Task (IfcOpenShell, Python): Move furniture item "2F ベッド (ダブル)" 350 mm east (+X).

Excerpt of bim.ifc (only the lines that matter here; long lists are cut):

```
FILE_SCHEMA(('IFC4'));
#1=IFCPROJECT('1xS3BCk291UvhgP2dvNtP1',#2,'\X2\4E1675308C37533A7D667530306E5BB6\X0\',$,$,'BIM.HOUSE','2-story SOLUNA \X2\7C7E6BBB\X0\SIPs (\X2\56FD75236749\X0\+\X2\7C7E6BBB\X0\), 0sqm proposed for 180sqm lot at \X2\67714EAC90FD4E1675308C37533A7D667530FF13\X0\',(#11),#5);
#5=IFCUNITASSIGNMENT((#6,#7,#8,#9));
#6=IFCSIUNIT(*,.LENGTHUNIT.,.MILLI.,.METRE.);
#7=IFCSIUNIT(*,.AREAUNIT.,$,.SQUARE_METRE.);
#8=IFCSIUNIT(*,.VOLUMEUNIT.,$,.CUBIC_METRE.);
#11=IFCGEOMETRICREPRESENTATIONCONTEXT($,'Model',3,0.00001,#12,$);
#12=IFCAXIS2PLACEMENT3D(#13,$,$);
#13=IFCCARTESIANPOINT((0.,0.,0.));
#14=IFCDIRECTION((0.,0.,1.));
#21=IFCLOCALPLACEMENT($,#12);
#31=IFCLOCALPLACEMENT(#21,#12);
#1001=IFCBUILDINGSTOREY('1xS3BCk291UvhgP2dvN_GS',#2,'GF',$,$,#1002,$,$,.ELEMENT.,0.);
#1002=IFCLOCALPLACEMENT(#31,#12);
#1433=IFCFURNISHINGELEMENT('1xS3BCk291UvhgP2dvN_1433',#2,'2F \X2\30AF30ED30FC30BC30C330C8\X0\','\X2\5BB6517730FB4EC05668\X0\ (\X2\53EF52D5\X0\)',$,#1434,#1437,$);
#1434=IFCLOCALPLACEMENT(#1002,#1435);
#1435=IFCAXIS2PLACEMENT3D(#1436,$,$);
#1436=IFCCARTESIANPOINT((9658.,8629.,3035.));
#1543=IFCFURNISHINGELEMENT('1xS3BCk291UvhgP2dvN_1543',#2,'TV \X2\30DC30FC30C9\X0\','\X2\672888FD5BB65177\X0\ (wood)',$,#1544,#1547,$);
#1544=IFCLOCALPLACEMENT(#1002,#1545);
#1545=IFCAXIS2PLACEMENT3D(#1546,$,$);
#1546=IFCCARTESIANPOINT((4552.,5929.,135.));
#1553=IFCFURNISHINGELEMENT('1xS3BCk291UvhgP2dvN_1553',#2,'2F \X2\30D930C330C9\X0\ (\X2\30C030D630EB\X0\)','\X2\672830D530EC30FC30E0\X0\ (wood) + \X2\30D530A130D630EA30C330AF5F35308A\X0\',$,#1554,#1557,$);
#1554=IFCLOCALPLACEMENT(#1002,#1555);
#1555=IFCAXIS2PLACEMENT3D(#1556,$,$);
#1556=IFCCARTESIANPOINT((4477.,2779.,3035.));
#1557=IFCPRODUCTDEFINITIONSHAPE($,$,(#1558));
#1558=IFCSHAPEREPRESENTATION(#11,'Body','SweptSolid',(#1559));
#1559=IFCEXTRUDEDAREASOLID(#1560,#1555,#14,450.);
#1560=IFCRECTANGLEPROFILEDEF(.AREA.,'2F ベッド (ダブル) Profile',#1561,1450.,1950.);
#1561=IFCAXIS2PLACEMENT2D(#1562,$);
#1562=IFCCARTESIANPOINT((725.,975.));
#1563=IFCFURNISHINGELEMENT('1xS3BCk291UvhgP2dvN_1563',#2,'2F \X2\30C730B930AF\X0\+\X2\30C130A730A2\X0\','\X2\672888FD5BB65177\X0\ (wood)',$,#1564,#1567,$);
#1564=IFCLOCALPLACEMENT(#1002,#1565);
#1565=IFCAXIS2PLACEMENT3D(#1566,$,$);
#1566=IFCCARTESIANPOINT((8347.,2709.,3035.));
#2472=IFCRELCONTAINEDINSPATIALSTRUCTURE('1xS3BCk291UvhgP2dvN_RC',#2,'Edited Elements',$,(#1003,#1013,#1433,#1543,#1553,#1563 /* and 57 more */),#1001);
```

```python
import ifcopenshell
import ifcopenshell.api.geometry
import ifcopenshell.util.placement
import ifcopenshell.util.unit

model = ifcopenshell.open("bim.ifc")
unit_scale = ifcopenshell.util.unit.calculate_unit_scale(model)

item = model.by_id(1553)
matrix = ifcopenshell.util.placement.get_local_placement(item.ObjectPlacement)
matrix[0, 3] += 0.35 / unit_scale
ifcopenshell.api.geometry.edit_object_placement(model, product=item, matrix=matrix, is_si=False)

print(ifcopenshell.util.placement.get_local_placement(item.ObjectPlacement).round(3) + 0.0)

model.write("bim_edited.ifc")
```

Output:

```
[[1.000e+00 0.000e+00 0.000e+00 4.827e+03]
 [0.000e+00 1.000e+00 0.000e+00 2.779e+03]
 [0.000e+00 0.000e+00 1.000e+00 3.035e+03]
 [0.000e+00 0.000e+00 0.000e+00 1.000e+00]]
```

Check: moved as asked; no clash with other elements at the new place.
